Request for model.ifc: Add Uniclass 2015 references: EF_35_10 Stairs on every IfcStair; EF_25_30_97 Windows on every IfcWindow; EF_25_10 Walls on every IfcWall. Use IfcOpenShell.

First a look at what the model holds.

```python
import ifcopenshell

model = ifcopenshell.open("model.ifc")
print(model.schema)
print("classifications:", [c.Name for c in model.by_type("IfcClassification")])
for ifc_class in ("IfcDoor", "IfcRoof", "IfcStair", "IfcWall", "IfcWindow"):
    print(ifc_class, len(model.by_type(ifc_class)))
```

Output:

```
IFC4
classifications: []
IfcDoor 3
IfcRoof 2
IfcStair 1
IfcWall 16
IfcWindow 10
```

```python
import ifcopenshell
import ifcopenshell.api.classification

model = ifcopenshell.open("model.ifc")

system = ifcopenshell.api.classification.add_classification(model, classification="Uniclass 2015")

codes = {
    "IfcStair": ("EF_35_10", "Stairs"),
    "IfcWindow": ("EF_25_30_97", "Windows"),
    "IfcWall": ("EF_25_10", "Walls"),
}
for ifc_class, (code, name) in codes.items():
    products = model.by_type(ifc_class)
    ifcopenshell.api.classification.add_reference(
        model, products=products, classification=system, identification=code, name=name
    )
    print(code, len(products))

model.write("model_edited.ifc")
```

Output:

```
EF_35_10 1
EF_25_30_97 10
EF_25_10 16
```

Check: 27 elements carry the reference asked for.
